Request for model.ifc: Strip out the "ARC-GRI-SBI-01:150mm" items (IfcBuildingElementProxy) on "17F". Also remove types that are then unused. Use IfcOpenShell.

First a look at what the model holds.

```python
import ifcopenshell
import ifcopenshell.util.element

model = ifcopenshell.open("model.ifc")
print(model.schema)
storey = next(s for s in model.by_type("IfcBuildingStorey") if s.Name == "17F")
proxies = [e for e in ifcopenshell.util.element.get_decomposition(storey) if e.is_a("IfcBuildingElementProxy")]
seen = {}
for e in proxies:
    element_type = ifcopenshell.util.element.get_type(e)
    name = element_type.Name if element_type not in (None, e) else None
    seen[name] = seen.get(name, 0) + 1
for name, count in sorted(seen.items(), key=str):
    print(count, "x", name)
```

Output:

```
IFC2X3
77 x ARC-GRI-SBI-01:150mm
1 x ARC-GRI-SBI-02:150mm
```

```python
import ifcopenshell
import ifcopenshell.api.root
import ifcopenshell.util.element

model = ifcopenshell.open("model.ifc")

storey = next(s for s in model.by_type("IfcBuildingStorey") if s.Name == "17F")
proxies = [e for e in ifcopenshell.util.element.get_decomposition(storey) if e.is_a("IfcBuildingElementProxy")]
targets = [e for e in proxies if (t := ifcopenshell.util.element.get_type(e)) not in (None, e) and t.Name == "ARC-GRI-SBI-01:150mm"]
types = {ifcopenshell.util.element.get_type(e) for e in targets} - {None, *targets}

for e in targets:
    ifcopenshell.api.root.remove_product(model, product=e)
print(len(targets), "removed")

unused = [t for t in types if not ifcopenshell.util.element.get_types(t)]
for t in unused:
    ifcopenshell.api.root.remove_product(model, product=t)
print(len(unused), "unused types removed")

model.write("model-out.ifc")
```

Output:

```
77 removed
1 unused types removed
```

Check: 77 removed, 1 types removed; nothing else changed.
